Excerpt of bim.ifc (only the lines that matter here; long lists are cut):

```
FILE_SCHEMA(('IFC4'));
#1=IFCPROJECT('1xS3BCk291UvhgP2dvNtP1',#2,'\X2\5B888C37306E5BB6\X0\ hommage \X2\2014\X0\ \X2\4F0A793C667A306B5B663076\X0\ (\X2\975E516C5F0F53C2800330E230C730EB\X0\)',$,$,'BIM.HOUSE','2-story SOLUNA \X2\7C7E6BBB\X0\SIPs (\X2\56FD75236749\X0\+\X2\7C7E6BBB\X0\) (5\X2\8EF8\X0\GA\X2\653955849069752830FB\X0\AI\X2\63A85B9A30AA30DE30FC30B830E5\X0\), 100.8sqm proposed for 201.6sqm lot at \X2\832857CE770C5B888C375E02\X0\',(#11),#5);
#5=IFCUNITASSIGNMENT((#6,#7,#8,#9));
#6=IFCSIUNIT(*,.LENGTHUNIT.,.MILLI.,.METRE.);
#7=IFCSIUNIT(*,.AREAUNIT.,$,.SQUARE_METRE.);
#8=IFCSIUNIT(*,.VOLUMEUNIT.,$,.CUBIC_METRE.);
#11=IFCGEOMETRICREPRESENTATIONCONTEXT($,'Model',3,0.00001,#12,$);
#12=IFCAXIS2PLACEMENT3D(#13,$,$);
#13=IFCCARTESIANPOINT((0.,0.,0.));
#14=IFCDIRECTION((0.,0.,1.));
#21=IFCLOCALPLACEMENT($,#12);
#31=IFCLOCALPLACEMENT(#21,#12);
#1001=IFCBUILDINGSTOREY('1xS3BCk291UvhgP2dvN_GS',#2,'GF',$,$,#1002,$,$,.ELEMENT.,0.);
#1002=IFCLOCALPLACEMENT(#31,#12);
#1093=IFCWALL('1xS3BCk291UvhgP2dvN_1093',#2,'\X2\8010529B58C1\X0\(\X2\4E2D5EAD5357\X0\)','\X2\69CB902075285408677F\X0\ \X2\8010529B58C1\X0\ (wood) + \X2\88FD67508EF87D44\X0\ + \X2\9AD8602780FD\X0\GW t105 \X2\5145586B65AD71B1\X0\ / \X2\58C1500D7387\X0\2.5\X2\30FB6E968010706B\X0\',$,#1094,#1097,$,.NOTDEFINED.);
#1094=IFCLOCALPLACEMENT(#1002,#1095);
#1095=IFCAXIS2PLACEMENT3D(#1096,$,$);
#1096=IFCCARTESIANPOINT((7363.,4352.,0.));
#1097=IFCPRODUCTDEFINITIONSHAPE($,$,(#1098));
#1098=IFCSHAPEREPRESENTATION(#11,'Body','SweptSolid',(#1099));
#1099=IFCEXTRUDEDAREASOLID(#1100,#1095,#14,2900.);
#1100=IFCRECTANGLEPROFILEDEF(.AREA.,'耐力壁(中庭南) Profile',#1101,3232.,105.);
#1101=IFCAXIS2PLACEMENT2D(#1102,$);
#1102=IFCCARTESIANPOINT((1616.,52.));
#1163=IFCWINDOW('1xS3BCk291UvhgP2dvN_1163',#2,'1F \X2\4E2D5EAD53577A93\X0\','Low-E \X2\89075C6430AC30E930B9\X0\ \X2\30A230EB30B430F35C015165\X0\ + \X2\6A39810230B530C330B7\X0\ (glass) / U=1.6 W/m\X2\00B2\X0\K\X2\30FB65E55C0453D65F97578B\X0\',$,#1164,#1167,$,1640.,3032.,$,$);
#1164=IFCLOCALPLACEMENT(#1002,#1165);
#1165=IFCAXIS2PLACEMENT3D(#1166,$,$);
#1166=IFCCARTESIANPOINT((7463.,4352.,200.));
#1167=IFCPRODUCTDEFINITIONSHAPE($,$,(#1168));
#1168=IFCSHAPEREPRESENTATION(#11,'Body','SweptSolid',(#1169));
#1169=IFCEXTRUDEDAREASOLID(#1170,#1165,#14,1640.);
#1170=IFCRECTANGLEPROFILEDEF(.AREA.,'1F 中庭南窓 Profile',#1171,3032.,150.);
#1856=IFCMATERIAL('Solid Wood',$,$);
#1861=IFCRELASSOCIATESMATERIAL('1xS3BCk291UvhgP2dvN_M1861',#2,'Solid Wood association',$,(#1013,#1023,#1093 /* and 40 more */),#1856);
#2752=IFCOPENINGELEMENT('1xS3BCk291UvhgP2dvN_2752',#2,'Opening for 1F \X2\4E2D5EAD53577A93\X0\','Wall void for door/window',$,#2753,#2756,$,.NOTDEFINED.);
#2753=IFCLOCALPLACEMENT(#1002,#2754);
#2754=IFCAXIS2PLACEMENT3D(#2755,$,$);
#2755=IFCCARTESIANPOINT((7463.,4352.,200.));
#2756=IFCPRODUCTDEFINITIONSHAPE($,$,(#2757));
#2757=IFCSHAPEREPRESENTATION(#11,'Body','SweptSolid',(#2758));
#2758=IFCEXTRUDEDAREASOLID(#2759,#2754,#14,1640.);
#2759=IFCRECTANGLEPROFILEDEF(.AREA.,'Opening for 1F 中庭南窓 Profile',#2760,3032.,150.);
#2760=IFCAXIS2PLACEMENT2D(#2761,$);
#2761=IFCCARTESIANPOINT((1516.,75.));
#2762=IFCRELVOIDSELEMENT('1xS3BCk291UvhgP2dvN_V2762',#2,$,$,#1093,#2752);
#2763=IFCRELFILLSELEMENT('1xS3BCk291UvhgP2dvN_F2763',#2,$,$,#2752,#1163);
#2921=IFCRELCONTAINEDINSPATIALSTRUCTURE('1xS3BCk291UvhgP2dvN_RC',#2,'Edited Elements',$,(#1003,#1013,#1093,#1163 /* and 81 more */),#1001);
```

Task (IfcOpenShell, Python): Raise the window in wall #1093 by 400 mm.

```python
import numpy as np
import ifcopenshell
import ifcopenshell.api.geometry
import ifcopenshell.util.placement
import ifcopenshell.util.unit

model = ifcopenshell.open("bim.ifc")
unit_scale = ifcopenshell.util.unit.calculate_unit_scale(model)

window = model.by_id(1163)
opening = window.FillsVoids[0].RelatingOpeningElement
dz = 400.0

shift = np.array([0.0, 0.0, dz])
# The window is not placed relative to its opening, so move both.
for product in (opening, window):
    matrix = ifcopenshell.util.placement.get_local_placement(product.ObjectPlacement)
    matrix[:3, 3] += shift
    ifcopenshell.api.geometry.edit_object_placement(model, product=product, matrix=matrix, is_si=False)

print(f"moved by {dz * unit_scale:+.3f} m")

model.write("bim_rev.ifc")
```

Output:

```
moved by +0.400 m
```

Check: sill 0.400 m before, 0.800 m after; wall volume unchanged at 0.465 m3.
